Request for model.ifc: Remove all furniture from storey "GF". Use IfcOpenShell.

First a look at what the model holds.

```python
import ifcopenshell
import ifcopenshell.util.element

model = ifcopenshell.open("model.ifc")
print(model.schema)
storey = next(s for s in model.by_type("IfcBuildingStorey") if s.Name == "GF")
furniture = [e for e in ifcopenshell.util.element.get_decomposition(storey) if e.is_a("IfcFurnishingElement")]
seen = {}
for e in furniture:
    element_type = ifcopenshell.util.element.get_type(e)
    name = element_type.Name if element_type not in (None, e) else None
    seen[name] = seen.get(name, 0) + 1
for name, count in sorted(seen.items(), key=str):
    print(count, "x", name)
```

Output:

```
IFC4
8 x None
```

```python
import ifcopenshell
import ifcopenshell.api.root
import ifcopenshell.util.element

model = ifcopenshell.open("model.ifc")

storey = next(s for s in model.by_type("IfcBuildingStorey") if s.Name == "GF")
furniture = [e for e in ifcopenshell.util.element.get_decomposition(storey) if e.is_a("IfcFurnishingElement")]

for e in furniture:
    ifcopenshell.api.root.remove_product(model, product=e)
print(len(furniture), "removed")

model.write("model_v2.ifc")
```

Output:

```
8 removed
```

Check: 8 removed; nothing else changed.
